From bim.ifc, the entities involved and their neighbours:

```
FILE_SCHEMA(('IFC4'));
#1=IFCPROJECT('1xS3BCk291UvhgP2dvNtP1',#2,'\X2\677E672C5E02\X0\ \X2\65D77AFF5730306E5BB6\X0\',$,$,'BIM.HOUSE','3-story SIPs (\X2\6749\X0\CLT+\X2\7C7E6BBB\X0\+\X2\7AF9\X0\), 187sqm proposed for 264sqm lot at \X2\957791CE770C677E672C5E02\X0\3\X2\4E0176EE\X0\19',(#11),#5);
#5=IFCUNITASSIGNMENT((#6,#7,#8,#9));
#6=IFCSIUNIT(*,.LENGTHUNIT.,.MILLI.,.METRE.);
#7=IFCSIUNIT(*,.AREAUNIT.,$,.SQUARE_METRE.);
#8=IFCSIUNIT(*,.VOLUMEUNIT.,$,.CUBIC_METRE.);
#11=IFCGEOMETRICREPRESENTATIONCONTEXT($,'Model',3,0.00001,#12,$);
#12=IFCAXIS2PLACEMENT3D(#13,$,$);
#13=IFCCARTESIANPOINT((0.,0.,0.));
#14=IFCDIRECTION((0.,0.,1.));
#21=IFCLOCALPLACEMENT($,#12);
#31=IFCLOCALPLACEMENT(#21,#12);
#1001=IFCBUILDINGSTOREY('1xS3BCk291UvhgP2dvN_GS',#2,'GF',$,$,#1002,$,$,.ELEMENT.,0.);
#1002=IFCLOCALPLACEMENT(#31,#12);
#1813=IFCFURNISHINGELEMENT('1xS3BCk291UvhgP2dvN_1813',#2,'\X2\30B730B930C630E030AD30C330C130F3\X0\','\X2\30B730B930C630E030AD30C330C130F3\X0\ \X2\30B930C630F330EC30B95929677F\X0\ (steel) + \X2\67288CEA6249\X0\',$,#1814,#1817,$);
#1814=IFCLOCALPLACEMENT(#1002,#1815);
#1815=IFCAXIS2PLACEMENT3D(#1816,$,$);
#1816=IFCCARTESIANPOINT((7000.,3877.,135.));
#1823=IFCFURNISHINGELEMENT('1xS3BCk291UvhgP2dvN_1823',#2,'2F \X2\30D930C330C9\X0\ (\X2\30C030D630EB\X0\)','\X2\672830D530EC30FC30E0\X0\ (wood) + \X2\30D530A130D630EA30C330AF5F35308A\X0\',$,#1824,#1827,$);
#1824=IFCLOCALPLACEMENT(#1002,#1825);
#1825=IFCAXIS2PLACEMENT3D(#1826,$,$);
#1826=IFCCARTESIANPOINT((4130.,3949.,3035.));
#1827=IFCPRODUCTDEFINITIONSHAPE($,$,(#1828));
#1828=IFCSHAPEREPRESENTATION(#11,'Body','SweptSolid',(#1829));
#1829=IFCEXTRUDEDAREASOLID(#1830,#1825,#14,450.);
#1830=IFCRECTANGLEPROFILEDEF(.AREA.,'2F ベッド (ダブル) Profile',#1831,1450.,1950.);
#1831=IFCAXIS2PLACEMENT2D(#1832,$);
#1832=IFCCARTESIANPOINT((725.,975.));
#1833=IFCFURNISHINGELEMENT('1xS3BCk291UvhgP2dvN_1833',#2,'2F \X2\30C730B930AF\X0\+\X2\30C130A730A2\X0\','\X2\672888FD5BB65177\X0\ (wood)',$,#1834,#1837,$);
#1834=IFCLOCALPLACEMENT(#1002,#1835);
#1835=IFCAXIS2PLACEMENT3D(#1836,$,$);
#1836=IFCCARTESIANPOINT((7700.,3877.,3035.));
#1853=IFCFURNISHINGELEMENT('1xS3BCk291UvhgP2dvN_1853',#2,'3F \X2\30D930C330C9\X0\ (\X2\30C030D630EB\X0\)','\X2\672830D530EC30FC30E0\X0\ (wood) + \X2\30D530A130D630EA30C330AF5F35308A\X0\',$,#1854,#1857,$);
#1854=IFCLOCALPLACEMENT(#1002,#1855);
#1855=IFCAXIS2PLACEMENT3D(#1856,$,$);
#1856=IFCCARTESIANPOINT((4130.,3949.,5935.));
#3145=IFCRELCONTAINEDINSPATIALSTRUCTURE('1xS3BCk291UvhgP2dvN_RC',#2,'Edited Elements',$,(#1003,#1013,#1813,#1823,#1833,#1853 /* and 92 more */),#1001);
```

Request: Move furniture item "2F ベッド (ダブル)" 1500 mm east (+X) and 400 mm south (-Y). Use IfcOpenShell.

```python
import ifcopenshell
import ifcopenshell.api.geometry
import ifcopenshell.util.placement

model = ifcopenshell.open("bim.ifc")

item = model.by_id(1823)
matrix = ifcopenshell.util.placement.get_local_placement(item.ObjectPlacement)
matrix[0, 3] += 1500.0
matrix[1, 3] -= 400.0
ifcopenshell.api.geometry.edit_object_placement(model, product=item, matrix=matrix, is_si=False)

print(ifcopenshell.util.placement.get_local_placement(item.ObjectPlacement).round(3) + 0.0)

model.write("bim_edited.ifc")
```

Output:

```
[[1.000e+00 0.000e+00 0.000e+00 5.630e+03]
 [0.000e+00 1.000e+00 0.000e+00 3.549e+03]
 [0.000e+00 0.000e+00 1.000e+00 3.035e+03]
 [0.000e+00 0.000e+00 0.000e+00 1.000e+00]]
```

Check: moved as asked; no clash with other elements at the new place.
